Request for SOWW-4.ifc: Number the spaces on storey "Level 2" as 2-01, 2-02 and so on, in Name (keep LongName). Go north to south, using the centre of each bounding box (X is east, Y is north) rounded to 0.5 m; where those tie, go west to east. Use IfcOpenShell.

First a look at what the model holds.

```python
import ifcopenshell
import ifcopenshell.util.element
import ifcopenshell.util.placement

model = ifcopenshell.open("SOWW-4.ifc")
print(model.schema)
storey = next(s for s in model.by_type("IfcBuildingStorey") if s.Name == "Level 2")
spaces = [e for e in ifcopenshell.util.element.get_decomposition(storey) if e.is_a("IfcSpace")]
for e in sorted(spaces, key=lambda e: e.id()):
    origin = ifcopenshell.util.placement.get_local_placement(e.ObjectPlacement)[:3, 3]
    print(e.id(), e.Name, e.LongName, origin.round(2) + 0.0, sep=" | ")
```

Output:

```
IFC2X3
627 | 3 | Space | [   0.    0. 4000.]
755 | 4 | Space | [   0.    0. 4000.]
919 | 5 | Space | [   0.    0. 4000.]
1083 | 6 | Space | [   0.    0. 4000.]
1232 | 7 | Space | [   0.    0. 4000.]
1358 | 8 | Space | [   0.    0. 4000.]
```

```python
import ifcopenshell
import ifcopenshell.geom
import ifcopenshell.util.element
import ifcopenshell.util.shape

model = ifcopenshell.open("SOWW-4.ifc")
settings = ifcopenshell.geom.settings()
settings.set("use-world-coords", True)


def centre(element):
    shape = ifcopenshell.geom.create_shape(settings, element)
    return ifcopenshell.util.shape.get_bbox_centroid(shape.geometry)


storey = next(s for s in model.by_type("IfcBuildingStorey") if s.Name == "Level 2")
spaces = [e for e in ifcopenshell.util.element.get_decomposition(storey) if e.is_a("IfcSpace")]

# Insertion points can sit at a corner or the storey origin, so sort by the geometry (in metres).
centres = {e: centre(e) for e in spaces}
spaces.sort(key=lambda e: (-round(centres[e][1] / 0.5), centres[e][0]))

for i, e in enumerate(spaces, start=1):
    number = f"2-{i:02d}"
    e.Name = number
    print(e.id(), number)

model.write("SOWW-4_edited.ifc")
```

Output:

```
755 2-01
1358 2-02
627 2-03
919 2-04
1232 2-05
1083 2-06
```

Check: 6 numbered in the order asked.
